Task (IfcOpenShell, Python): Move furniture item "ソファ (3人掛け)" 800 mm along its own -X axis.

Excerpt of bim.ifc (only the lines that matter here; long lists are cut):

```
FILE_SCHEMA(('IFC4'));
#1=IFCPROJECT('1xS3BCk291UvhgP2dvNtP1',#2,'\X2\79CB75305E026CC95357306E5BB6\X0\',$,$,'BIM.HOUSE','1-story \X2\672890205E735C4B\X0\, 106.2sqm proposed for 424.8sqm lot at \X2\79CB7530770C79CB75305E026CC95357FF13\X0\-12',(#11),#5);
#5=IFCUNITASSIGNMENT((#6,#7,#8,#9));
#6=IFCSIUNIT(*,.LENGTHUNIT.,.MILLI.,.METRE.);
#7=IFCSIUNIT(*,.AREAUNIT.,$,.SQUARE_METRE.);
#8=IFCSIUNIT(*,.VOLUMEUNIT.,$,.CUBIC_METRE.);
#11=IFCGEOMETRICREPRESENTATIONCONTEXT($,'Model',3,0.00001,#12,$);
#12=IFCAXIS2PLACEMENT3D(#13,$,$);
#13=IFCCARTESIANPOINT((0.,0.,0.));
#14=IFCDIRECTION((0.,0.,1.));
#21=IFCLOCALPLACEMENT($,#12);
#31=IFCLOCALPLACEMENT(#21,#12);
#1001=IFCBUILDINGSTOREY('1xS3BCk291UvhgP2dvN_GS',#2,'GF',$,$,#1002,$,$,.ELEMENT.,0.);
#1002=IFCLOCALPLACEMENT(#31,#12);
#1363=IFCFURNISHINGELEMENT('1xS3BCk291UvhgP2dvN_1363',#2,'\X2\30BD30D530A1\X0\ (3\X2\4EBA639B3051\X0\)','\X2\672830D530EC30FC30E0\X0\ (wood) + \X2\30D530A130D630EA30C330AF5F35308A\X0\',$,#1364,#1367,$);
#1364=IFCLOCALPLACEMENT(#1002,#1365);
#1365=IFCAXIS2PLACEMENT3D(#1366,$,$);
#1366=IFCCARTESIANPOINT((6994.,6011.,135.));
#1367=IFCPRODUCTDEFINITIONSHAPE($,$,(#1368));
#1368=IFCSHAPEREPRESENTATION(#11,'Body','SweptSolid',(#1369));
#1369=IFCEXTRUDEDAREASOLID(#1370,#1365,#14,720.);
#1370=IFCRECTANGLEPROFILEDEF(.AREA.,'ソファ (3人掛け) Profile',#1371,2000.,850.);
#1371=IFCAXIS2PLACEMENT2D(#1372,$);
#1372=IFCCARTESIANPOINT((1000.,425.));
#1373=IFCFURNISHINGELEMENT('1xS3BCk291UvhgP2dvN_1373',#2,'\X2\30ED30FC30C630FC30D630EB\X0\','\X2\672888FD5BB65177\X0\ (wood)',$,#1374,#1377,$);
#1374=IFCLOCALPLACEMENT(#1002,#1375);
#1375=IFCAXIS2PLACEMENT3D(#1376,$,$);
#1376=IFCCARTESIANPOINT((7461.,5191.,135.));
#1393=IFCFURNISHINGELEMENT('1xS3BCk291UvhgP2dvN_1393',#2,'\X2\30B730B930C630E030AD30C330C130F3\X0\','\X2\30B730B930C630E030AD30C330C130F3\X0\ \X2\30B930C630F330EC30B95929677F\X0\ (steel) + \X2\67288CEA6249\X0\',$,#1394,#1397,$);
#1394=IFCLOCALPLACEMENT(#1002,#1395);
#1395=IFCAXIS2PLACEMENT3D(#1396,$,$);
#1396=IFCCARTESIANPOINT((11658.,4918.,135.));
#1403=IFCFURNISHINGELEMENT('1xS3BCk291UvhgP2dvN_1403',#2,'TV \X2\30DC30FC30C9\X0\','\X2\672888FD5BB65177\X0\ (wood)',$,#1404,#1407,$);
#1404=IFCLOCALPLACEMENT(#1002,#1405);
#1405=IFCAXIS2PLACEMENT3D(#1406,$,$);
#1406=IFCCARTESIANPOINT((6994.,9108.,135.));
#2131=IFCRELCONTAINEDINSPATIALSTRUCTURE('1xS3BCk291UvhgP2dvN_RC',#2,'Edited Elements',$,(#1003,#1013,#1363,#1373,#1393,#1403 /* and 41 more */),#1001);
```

```python
import ifcopenshell
import ifcopenshell.api.geometry
import ifcopenshell.util.placement

model = ifcopenshell.open("bim.ifc")

item = model.by_guid("1xS3BCk291UvhgP2dvN_1363")
matrix = ifcopenshell.util.placement.get_local_placement(item.ObjectPlacement)
matrix[:3, 3] -= matrix[:3, 0] * 800.0
ifcopenshell.api.geometry.edit_object_placement(model, product=item, matrix=matrix, is_si=False)

print(ifcopenshell.util.placement.get_local_placement(item.ObjectPlacement).round(3) + 0.0)

model.write("bim_edited.ifc")
```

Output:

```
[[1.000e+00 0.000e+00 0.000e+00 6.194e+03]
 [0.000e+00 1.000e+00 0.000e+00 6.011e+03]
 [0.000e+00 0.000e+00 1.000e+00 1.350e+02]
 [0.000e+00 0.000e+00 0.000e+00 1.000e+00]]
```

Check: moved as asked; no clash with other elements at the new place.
